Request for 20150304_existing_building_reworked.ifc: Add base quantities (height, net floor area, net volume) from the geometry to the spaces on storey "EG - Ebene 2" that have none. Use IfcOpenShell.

First a look at what the model holds.

```python
import ifcopenshell
import ifcopenshell.util.element
import ifcopenshell.util.unit

model = ifcopenshell.open("20150304_existing_building_reworked.ifc")
print(model.schema)
for unit_type in ("LENGTHUNIT", "AREAUNIT", "VOLUMEUNIT"):
    print(unit_type, ifcopenshell.util.unit.calculate_unit_scale(model, unit_type))
storey = next(s for s in model.by_type("IfcBuildingStorey") if s.Name == "EG - Ebene 2")
spaces = [e for e in ifcopenshell.util.element.get_decomposition(storey) if e.is_a("IfcSpace")]
for e in sorted(spaces, key=lambda e: e.id()):
    print(e.id(), e.is_a(), e.Name, list(ifcopenshell.util.element.get_psets(e, qtos_only=True)), sep=" | ")
```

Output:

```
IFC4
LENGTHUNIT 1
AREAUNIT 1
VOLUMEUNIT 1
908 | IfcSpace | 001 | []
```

```python
import ifcopenshell
import ifcopenshell.api.pset
import ifcopenshell.geom
import ifcopenshell.util.element
import ifcopenshell.util.shape
import ifcopenshell.util.unit

model = ifcopenshell.open("20150304_existing_building_reworked.ifc")
unit_scale = ifcopenshell.util.unit.calculate_unit_scale(model)
area_scale = ifcopenshell.util.unit.calculate_unit_scale(model, "AREAUNIT")
volume_scale = ifcopenshell.util.unit.calculate_unit_scale(model, "VOLUMEUNIT")
settings = ifcopenshell.geom.settings()

storey = next(s for s in model.by_type("IfcBuildingStorey") if s.Name == "EG - Ebene 2")
spaces = [e for e in ifcopenshell.util.element.get_decomposition(storey) if e.is_a("IfcSpace")]

for e in sorted(spaces, key=lambda e: e.id()):
    if ifcopenshell.util.element.get_psets(e, qtos_only=True, should_inherit=False):
        continue
    # Geometry comes back in metres, in the element's own axes.
    shape = ifcopenshell.geom.create_shape(settings, e)
    values = {
        "Height": ifcopenshell.util.shape.get_z(shape.geometry) / unit_scale,
        "NetFloorArea": ifcopenshell.util.shape.get_footprint_area(shape.geometry) / area_scale,
        "NetVolume": ifcopenshell.util.shape.get_volume(shape.geometry) / volume_scale,
    }
    qto = ifcopenshell.api.pset.add_qto(model, product=e, name="Qto_SpaceBaseQuantities")
    ifcopenshell.api.pset.edit_qto(model, qto=qto, properties=values)
    print(e.id(), {k: round(v, 3) for k, v in values.items()})

model.write("20150304_existing_building_reworked_edited.ifc")
```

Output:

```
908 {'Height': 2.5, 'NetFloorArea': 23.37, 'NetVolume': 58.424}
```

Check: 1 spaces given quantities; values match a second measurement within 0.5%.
